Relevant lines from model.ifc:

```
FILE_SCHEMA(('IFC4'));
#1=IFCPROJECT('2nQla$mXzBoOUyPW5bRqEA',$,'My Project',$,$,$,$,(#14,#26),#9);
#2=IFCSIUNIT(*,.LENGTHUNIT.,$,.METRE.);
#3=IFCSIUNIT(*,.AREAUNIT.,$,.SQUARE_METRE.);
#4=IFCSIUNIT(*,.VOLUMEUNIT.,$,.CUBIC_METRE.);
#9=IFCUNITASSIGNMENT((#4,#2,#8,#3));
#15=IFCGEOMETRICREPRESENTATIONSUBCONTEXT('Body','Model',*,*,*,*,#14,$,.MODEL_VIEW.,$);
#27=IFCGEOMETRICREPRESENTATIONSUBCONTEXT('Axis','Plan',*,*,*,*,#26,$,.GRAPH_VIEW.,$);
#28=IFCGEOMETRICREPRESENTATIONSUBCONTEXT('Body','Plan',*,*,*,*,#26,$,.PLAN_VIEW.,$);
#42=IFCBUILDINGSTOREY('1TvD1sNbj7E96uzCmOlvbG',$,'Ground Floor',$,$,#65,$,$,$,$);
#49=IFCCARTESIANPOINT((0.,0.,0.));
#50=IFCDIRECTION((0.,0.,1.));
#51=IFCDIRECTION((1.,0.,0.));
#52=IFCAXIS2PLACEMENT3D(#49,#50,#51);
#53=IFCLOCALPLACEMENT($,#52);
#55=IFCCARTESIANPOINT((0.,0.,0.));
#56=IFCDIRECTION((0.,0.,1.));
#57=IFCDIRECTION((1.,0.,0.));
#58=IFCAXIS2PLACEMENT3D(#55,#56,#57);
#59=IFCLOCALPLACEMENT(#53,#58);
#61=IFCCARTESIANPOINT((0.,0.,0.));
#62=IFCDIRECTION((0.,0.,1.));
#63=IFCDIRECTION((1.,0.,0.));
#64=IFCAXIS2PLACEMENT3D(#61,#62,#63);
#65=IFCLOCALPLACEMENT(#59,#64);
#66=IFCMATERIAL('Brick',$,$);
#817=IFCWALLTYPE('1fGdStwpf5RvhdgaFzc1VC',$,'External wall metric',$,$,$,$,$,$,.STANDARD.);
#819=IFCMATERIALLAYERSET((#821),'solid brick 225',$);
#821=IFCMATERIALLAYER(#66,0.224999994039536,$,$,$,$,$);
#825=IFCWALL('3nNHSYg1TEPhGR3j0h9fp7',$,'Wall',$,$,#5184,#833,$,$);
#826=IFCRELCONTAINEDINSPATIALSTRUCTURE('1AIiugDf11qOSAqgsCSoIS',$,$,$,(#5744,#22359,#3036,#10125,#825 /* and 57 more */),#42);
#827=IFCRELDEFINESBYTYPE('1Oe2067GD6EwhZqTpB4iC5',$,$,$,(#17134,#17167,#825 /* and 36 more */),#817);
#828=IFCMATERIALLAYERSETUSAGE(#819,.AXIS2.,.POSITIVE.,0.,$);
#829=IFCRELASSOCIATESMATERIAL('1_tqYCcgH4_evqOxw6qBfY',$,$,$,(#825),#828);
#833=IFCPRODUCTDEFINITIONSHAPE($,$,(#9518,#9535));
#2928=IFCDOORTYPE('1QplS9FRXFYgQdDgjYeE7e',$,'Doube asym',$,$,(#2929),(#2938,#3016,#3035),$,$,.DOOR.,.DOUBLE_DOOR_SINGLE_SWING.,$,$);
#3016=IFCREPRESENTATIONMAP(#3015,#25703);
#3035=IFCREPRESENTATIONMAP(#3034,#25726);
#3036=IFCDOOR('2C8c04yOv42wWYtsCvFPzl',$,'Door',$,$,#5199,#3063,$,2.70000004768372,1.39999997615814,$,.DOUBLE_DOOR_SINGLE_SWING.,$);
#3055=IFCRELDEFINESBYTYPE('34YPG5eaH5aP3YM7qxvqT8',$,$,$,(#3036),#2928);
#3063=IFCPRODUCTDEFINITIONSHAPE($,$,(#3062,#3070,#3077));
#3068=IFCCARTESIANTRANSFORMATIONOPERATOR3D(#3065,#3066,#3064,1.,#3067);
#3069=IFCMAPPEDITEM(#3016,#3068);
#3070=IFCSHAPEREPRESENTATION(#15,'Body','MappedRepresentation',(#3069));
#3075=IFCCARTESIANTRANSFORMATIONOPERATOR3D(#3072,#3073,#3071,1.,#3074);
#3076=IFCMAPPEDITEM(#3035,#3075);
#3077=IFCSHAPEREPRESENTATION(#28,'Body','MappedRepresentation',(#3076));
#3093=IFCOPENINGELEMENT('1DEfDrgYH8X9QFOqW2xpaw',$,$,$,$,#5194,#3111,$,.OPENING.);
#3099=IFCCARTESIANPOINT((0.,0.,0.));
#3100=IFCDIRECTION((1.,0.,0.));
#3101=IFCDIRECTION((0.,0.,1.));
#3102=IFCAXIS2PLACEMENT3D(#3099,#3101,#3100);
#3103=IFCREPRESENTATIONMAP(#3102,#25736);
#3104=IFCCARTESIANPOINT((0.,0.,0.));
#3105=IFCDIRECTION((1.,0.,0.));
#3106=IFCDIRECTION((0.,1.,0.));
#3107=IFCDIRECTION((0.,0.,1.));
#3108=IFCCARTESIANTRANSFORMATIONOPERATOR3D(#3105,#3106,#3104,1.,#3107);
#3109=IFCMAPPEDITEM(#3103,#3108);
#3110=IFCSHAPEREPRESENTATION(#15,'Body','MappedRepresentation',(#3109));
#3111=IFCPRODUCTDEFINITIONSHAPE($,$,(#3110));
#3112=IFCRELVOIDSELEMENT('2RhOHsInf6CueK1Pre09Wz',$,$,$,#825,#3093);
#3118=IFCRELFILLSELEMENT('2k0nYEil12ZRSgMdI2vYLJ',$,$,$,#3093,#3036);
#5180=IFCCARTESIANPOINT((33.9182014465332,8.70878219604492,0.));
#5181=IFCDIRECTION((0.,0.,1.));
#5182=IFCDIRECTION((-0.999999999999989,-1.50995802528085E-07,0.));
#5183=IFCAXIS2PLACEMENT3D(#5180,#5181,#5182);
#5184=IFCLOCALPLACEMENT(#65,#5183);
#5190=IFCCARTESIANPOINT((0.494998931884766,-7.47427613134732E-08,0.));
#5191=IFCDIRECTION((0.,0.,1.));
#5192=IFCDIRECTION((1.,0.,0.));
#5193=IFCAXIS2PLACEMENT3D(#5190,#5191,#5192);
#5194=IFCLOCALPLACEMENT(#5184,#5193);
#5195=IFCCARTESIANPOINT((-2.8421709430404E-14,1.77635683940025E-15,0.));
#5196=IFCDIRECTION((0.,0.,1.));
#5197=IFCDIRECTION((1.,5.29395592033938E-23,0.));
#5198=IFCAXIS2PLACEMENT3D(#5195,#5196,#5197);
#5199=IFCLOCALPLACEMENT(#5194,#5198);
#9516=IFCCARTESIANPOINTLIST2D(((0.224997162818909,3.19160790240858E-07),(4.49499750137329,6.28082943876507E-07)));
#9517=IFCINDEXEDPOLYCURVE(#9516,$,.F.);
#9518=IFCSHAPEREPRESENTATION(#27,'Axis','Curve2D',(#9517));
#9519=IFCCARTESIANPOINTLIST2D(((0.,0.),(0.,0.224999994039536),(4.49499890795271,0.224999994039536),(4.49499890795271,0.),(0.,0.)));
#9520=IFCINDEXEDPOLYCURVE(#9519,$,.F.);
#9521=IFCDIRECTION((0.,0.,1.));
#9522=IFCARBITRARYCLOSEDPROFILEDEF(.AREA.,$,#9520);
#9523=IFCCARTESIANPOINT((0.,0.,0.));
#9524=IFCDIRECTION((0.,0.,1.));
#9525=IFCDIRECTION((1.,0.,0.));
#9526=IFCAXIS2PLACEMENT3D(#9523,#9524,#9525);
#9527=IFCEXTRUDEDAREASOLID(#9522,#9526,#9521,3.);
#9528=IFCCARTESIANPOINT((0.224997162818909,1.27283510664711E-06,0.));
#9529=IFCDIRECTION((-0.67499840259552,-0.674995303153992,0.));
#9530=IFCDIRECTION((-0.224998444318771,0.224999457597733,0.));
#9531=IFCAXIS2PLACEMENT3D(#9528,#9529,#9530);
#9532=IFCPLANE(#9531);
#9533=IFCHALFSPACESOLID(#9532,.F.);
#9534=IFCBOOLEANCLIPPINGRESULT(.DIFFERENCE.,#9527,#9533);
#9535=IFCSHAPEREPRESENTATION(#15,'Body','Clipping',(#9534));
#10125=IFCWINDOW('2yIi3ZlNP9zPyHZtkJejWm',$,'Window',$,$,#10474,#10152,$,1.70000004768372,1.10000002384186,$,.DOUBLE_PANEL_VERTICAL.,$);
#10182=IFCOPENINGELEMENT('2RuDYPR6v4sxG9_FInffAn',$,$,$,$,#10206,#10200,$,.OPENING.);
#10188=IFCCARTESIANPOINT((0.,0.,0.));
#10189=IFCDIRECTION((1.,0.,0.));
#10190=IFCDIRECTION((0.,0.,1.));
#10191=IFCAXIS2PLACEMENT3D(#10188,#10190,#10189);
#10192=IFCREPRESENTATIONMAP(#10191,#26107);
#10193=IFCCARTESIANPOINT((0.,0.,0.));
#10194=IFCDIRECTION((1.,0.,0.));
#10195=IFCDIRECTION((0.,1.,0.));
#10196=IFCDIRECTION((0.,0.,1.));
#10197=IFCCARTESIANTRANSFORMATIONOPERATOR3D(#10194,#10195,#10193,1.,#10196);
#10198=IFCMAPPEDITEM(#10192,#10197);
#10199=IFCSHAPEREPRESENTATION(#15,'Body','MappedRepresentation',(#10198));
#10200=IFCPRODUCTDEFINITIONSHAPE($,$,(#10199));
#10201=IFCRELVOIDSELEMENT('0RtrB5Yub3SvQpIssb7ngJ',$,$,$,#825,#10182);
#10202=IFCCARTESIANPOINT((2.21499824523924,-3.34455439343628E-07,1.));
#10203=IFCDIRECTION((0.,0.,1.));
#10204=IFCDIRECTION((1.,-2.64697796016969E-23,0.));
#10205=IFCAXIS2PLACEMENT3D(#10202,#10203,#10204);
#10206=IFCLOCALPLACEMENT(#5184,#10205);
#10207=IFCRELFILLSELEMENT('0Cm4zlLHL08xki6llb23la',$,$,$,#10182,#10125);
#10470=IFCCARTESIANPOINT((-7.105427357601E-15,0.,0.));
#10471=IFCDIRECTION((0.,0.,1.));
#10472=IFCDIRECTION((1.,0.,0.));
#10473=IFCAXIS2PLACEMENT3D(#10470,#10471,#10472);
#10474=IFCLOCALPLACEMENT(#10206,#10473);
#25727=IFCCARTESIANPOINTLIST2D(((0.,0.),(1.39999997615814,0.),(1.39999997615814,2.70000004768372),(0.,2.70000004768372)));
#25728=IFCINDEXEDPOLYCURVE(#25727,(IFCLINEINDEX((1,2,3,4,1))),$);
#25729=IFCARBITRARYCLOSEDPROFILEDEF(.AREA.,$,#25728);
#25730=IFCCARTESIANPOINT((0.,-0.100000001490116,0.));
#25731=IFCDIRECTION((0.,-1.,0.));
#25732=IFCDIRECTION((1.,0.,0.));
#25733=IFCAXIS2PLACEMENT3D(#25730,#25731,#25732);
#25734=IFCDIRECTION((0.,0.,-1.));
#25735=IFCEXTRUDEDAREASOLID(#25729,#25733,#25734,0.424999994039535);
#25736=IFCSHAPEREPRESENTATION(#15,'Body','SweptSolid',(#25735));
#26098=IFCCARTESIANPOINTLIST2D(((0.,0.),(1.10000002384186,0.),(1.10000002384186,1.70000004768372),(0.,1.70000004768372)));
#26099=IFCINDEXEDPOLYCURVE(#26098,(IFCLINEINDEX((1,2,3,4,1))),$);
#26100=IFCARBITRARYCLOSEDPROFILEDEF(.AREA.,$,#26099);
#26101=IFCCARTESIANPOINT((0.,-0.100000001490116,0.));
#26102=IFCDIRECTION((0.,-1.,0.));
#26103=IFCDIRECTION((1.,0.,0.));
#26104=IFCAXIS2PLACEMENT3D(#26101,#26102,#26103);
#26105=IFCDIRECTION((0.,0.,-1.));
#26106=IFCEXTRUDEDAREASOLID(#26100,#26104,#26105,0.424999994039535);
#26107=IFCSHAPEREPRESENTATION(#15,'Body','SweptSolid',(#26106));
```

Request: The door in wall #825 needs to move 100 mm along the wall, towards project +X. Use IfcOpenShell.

```python
import ifcopenshell
import ifcopenshell.api.geometry
import ifcopenshell.util.placement
import ifcopenshell.util.unit

model = ifcopenshell.open("model.ifc")
unit_scale = ifcopenshell.util.unit.calculate_unit_scale(model)

door = model.by_guid("2C8c04yOv42wWYtsCvFPzl")
opening = door.FillsVoids[0].RelatingOpeningElement
wall = opening.VoidsElements[0].RelatingBuildingElement

wall_matrix = ifcopenshell.util.placement.get_local_placement(wall.ObjectPlacement)
shift = wall_matrix[:3, 0] * -0.1 / unit_scale
before = ifcopenshell.util.placement.get_local_placement(door.ObjectPlacement)[:3, 3].copy()

# The door is placed relative to its opening, so it follows when the opening moves.
matrix = ifcopenshell.util.placement.get_local_placement(opening.ObjectPlacement)
matrix[:3, 3] += shift
ifcopenshell.api.geometry.edit_object_placement(
    model, product=opening, matrix=matrix, is_si=False, should_transform_children=True
)

after = ifcopenshell.util.placement.get_local_placement(door.ObjectPlacement)[:3, 3]
print("door moved by", (after - before).round(3) + 0.0)

model.write("model_rev.ifc")
```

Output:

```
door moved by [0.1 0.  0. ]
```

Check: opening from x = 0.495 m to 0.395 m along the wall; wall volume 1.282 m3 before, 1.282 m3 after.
